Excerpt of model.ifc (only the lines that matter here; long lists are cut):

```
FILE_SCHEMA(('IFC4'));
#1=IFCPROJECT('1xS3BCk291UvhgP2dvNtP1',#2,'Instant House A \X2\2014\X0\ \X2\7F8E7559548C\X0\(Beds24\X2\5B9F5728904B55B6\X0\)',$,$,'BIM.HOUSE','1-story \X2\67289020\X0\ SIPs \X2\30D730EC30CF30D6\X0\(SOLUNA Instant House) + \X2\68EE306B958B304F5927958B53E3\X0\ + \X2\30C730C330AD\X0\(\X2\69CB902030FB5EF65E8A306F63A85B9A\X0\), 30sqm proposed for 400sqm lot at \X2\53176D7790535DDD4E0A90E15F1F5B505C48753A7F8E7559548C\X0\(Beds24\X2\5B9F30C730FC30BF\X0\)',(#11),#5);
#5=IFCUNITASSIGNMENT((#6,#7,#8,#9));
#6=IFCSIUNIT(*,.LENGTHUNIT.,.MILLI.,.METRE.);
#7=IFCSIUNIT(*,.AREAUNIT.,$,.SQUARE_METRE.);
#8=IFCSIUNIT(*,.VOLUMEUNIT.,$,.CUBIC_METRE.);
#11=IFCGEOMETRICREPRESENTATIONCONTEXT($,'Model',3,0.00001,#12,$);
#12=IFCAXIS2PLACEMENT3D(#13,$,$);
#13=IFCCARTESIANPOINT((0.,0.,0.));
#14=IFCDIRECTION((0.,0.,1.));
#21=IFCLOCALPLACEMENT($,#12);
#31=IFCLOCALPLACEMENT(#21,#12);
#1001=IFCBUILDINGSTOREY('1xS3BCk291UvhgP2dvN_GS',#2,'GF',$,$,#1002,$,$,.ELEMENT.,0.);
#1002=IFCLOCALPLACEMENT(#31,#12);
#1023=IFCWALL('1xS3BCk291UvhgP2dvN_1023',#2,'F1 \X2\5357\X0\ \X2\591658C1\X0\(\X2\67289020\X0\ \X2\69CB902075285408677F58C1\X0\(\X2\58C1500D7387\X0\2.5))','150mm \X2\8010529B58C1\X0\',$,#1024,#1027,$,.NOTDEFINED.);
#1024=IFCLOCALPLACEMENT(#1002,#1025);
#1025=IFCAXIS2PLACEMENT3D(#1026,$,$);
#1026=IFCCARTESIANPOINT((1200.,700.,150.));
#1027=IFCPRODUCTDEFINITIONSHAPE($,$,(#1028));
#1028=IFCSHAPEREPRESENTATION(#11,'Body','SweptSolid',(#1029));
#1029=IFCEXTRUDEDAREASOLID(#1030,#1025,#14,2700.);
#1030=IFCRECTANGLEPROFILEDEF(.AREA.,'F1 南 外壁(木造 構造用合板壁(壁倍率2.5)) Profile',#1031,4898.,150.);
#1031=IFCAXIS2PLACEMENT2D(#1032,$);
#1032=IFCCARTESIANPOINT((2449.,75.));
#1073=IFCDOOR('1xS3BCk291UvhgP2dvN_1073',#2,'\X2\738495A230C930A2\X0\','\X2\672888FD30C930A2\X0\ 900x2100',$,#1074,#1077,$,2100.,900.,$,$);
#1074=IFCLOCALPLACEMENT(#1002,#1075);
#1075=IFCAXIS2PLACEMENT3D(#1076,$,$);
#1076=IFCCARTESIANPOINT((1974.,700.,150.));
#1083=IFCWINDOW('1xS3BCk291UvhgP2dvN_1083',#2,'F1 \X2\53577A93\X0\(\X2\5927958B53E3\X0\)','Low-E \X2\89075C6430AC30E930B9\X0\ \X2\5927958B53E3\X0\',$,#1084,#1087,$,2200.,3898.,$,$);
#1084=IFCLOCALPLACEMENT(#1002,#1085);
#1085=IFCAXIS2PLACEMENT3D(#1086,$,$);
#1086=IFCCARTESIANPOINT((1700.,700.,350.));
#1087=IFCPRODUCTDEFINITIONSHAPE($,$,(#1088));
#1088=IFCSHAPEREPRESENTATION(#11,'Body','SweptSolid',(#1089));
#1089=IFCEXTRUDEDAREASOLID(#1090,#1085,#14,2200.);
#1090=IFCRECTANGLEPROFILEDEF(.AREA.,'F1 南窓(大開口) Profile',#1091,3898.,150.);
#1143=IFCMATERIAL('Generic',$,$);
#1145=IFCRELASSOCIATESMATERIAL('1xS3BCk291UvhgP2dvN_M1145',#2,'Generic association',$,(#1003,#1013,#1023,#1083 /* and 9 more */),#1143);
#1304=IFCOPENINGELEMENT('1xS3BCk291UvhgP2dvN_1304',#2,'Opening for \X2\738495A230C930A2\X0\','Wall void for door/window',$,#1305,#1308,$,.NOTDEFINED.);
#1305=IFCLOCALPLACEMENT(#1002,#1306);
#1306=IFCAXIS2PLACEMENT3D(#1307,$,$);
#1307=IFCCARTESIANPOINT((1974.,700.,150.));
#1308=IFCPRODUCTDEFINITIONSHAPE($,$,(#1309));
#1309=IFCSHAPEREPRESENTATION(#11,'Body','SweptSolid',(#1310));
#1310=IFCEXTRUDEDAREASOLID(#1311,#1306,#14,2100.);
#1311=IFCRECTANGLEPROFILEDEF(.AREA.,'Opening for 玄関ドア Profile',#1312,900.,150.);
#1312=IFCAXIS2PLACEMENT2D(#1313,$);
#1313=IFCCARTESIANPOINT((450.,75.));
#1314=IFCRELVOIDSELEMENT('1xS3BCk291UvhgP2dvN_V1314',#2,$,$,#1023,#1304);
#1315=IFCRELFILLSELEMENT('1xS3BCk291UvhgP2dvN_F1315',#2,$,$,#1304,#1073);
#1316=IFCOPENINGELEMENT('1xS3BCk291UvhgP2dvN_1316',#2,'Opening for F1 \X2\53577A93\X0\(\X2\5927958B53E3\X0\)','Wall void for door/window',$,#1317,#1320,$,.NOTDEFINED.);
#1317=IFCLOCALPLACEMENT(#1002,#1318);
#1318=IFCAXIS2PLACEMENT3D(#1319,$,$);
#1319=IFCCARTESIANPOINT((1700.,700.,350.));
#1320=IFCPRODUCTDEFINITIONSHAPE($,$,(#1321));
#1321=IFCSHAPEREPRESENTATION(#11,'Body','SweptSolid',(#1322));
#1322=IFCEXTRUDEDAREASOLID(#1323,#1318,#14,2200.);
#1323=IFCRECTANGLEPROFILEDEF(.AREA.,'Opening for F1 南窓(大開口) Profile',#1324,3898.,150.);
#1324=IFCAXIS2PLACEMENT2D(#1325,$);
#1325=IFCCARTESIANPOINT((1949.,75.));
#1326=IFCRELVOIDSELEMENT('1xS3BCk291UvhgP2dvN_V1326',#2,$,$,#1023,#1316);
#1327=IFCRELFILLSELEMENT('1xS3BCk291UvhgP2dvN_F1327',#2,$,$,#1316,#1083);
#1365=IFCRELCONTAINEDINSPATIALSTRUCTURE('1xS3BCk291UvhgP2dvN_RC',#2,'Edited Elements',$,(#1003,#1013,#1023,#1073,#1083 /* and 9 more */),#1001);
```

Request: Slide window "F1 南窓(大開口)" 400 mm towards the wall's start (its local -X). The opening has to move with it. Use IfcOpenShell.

```python
import ifcopenshell
import ifcopenshell.api.geometry
import ifcopenshell.util.placement
import ifcopenshell.util.unit

model = ifcopenshell.open("model.ifc")
unit_scale = ifcopenshell.util.unit.calculate_unit_scale(model)

window = model.by_id(1083)
opening = window.FillsVoids[0].RelatingOpeningElement
wall = opening.VoidsElements[0].RelatingBuildingElement

wall_matrix = ifcopenshell.util.placement.get_local_placement(wall.ObjectPlacement)
shift = wall_matrix[:3, 0] * -0.4 / unit_scale
before = ifcopenshell.util.placement.get_local_placement(window.ObjectPlacement)[:3, 3].copy()

# The window is not placed relative to its opening, so move both.
for product in (opening, window):
    matrix = ifcopenshell.util.placement.get_local_placement(product.ObjectPlacement)
    matrix[:3, 3] += shift
    ifcopenshell.api.geometry.edit_object_placement(model, product=product, matrix=matrix, is_si=False)

after = ifcopenshell.util.placement.get_local_placement(window.ObjectPlacement)[:3, 3]
print("window moved by", (after - before).round(3) + 0.0)

model.write("model_edited.ifc")
```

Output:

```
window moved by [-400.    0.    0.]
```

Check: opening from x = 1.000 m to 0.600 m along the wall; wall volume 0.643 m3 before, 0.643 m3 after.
